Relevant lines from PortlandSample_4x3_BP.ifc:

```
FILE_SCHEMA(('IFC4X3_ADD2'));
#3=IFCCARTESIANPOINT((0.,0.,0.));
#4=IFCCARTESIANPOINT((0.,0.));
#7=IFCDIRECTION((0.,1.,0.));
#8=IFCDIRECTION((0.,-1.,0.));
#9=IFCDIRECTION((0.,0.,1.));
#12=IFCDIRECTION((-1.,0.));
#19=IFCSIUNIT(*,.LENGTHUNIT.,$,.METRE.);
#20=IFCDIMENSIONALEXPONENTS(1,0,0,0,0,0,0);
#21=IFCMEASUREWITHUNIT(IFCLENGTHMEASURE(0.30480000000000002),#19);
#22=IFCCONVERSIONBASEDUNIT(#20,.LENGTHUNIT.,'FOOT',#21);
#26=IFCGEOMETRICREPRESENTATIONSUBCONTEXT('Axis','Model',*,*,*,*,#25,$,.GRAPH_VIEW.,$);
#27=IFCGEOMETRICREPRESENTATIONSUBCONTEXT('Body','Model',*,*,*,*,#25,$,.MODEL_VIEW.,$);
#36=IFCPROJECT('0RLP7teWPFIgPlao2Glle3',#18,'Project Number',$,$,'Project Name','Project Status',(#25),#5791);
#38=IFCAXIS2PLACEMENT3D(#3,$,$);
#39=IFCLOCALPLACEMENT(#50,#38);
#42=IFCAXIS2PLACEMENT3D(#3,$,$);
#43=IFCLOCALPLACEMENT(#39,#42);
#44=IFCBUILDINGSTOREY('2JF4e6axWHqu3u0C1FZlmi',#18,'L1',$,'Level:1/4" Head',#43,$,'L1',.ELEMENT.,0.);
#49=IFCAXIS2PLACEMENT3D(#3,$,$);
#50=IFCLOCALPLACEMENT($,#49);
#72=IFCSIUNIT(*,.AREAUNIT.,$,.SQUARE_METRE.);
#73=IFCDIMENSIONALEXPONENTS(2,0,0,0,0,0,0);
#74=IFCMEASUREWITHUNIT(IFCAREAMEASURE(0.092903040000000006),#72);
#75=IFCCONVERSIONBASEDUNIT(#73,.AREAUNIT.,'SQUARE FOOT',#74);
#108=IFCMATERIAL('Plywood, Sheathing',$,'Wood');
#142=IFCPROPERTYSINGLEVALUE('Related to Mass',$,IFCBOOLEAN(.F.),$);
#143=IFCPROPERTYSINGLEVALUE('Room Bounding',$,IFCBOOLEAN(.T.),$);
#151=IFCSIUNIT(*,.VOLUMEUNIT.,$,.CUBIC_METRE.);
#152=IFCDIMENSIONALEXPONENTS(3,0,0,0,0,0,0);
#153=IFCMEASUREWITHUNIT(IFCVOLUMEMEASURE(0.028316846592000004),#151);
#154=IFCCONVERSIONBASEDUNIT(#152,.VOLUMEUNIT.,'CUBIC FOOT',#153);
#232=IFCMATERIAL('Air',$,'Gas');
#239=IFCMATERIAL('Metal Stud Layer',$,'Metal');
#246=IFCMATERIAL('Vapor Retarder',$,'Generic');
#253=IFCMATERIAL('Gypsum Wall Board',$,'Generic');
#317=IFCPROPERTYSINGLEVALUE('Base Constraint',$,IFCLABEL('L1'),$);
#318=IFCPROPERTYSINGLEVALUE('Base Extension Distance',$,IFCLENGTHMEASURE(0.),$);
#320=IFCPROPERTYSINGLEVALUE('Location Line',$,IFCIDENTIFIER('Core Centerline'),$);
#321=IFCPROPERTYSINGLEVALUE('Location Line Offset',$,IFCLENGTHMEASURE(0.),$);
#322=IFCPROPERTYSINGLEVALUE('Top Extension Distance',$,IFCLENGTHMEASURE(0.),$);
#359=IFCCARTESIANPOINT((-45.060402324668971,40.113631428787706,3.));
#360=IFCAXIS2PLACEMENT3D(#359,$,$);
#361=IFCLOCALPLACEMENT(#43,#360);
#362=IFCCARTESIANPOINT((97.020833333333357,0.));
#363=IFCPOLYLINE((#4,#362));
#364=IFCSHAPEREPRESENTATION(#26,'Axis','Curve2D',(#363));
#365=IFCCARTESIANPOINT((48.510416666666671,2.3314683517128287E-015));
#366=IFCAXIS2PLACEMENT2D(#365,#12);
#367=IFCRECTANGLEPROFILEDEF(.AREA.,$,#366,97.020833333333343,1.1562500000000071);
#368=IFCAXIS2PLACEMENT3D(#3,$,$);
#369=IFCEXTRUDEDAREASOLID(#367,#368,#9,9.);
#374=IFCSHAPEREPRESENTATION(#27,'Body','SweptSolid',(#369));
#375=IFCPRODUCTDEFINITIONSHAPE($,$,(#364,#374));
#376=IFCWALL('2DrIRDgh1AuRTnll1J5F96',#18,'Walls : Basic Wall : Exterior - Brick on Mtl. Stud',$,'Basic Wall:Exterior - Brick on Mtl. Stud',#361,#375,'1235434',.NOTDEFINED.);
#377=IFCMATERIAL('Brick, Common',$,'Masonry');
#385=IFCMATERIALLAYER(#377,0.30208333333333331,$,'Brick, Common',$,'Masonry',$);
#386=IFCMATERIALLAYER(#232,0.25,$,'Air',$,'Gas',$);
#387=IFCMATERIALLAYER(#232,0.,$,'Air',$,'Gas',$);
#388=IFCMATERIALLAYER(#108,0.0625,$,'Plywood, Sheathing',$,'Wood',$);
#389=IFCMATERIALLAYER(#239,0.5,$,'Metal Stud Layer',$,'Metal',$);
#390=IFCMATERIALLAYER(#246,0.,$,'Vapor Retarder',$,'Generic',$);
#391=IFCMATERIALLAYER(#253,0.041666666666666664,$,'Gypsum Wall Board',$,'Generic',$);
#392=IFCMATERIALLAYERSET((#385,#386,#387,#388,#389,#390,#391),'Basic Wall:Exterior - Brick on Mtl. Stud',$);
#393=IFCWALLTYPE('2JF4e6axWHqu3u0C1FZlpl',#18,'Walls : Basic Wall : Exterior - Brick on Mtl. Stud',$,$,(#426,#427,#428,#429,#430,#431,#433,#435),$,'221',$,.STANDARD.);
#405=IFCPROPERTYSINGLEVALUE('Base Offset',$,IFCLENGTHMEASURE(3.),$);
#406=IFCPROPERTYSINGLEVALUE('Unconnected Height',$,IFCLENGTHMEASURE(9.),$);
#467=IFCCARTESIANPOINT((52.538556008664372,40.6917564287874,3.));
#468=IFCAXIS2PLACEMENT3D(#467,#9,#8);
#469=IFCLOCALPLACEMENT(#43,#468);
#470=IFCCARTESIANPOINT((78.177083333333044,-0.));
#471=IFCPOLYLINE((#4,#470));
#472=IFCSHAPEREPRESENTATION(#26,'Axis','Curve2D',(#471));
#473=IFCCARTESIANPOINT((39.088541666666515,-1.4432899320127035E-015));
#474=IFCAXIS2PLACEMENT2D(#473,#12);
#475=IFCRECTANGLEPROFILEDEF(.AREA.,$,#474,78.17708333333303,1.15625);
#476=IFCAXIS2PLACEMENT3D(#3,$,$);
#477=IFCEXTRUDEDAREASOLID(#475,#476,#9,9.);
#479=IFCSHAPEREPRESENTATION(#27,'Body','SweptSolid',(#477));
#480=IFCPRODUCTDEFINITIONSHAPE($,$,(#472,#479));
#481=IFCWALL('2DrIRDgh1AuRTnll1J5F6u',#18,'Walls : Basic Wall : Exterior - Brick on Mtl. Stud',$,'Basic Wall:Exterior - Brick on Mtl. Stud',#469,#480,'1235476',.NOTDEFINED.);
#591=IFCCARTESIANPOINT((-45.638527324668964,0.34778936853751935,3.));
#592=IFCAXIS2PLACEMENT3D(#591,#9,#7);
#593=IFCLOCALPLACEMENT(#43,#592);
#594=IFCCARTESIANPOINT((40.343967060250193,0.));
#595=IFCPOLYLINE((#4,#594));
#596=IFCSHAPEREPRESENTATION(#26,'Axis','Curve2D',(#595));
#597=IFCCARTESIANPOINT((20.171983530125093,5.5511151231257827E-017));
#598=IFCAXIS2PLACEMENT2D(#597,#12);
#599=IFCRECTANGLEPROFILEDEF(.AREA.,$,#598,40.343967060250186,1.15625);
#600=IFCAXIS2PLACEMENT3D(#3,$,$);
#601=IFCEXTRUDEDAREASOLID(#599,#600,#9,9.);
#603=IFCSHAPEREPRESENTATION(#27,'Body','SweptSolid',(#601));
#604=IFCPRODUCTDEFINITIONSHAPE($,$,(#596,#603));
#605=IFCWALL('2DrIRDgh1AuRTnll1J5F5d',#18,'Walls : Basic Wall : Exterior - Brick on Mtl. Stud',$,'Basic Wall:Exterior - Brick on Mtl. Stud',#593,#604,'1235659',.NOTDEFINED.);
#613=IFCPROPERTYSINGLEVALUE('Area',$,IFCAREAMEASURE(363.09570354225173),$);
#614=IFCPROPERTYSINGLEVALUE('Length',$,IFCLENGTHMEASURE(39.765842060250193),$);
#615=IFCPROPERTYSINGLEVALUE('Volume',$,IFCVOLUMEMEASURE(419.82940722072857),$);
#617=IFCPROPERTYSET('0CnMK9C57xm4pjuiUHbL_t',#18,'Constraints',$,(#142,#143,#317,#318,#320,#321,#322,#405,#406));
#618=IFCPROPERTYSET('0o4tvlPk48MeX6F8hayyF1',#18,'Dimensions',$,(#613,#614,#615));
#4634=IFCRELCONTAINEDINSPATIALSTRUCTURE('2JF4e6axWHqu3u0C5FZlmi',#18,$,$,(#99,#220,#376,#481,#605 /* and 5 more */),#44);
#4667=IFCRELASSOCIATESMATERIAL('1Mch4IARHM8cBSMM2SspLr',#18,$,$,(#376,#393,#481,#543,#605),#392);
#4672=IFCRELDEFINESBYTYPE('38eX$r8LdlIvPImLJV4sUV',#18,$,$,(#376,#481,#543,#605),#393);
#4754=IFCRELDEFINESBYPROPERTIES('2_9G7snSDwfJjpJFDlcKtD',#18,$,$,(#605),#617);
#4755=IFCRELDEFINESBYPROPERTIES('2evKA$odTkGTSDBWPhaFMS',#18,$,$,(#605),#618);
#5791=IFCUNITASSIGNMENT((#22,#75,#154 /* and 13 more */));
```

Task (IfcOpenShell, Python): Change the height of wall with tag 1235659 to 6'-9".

```python
import ifcopenshell
import ifcopenshell.api.pset
import ifcopenshell.geom
import ifcopenshell.util.element
import ifcopenshell.util.representation
import ifcopenshell.util.shape
import ifcopenshell.util.unit

model = ifcopenshell.open("PortlandSample_4x3_BP.ifc")
unit_scale = ifcopenshell.util.unit.calculate_unit_scale(model)
area_scale = ifcopenshell.util.unit.calculate_unit_scale(model, "AREAUNIT")
volume_scale = ifcopenshell.util.unit.calculate_unit_scale(model, "VOLUMEUNIT")
settings = ifcopenshell.geom.settings()


def volume(element):
    """Net volume in cubic metres, openings subtracted."""
    shape = ifcopenshell.geom.create_shape(settings, element)
    return ifcopenshell.util.shape.get_volume(shape.geometry)


wall = model.by_id(605)
before = volume(wall)

body = ifcopenshell.util.representation.get_representation(wall, "Model", "Body")
solid = body.Items[0]
old_height = solid.Depth
solid.Depth = 81 * 0.0254 / unit_scale
after = volume(wall)
thickness = 0.3524  # wall thickness in metres

# Update the stored height, areas and volumes.
pset = model.by_id(ifcopenshell.util.element.get_pset(wall, "Constraints", should_inherit=False)["id"])
ifcopenshell.api.pset.edit_pset(model, pset=pset, properties={
    "Unconnected Height": model.create_entity("IfcLengthMeasure", solid.Depth),
})
pset = model.by_id(ifcopenshell.util.element.get_pset(wall, "Dimensions", should_inherit=False)["id"])
ifcopenshell.api.pset.edit_pset(model, pset=pset, properties={
    "Area": model.create_entity("IfcAreaMeasure", after / thickness / area_scale),
    "Volume": model.create_entity("IfcVolumeMeasure", after / volume_scale),
})

print(f"height {old_height:g} -> {solid.Depth:g}, volume {before:.3f} -> {after:.3f} m3")

model.write("PortlandSample_4x3_BP_edited.ifc")
```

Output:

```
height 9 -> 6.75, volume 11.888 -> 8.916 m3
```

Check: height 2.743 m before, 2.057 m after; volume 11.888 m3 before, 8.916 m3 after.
